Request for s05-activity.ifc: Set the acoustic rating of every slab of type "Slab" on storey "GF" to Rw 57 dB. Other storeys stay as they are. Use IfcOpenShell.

First a look at what the model holds.

```python
import ifcopenshell
import ifcopenshell.util.element

model = ifcopenshell.open("s05-activity.ifc")
print(model.schema)
storey = next(s for s in model.by_type("IfcBuildingStorey") if s.Name == "GF")
slabs = [e for e in ifcopenshell.util.element.get_decomposition(storey) if e.is_a("IfcSlab")]
seen = {}
for e in slabs:
    element_type = ifcopenshell.util.element.get_type(e)
    key = (element_type.Name if element_type != e and element_type else None, ifcopenshell.util.element.get_pset(e, "Pset_SlabCommon", "AcousticRating"))
    seen[key] = seen.get(key, 0) + 1
for (name, value), count in sorted(seen.items(), key=str):
    print(count, "x", name, "|", value)
```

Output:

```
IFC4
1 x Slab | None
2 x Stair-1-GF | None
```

```python
import ifcopenshell
import ifcopenshell.api.pset
import ifcopenshell.util.element

model = ifcopenshell.open("s05-activity.ifc")

storey = next(s for s in model.by_type("IfcBuildingStorey") if s.Name == "GF")
slabs = [e for e in ifcopenshell.util.element.get_decomposition(storey) if e.is_a("IfcSlab")]

count = 0
for e in slabs:
    element_type = ifcopenshell.util.element.get_type(e)
    if element_type in (None, e) or element_type.Name != "Slab":
        continue
    # add_pset returns the element's existing set when there is one.
    pset = ifcopenshell.api.pset.add_pset(model, product=e, name="Pset_SlabCommon")
    ifcopenshell.api.pset.edit_pset(model, pset=pset, properties={"AcousticRating": "Rw 57 dB"})
    count += 1

print(count, "slabs updated")

model.write("s05-activity_v2.ifc")
```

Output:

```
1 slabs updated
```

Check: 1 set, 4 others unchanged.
